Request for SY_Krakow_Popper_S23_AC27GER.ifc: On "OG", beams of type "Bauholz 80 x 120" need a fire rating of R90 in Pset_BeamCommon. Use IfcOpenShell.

First a look at what the model holds.

```python
import ifcopenshell
import ifcopenshell.util.element

model = ifcopenshell.open("SY_Krakow_Popper_S23_AC27GER.ifc")
print(model.schema)
storey = next(s for s in model.by_type("IfcBuildingStorey") if s.Name == "OG")
beams = [e for e in ifcopenshell.util.element.get_decomposition(storey) if e.is_a("IfcBeam")]
seen = {}
for e in beams:
    element_type = ifcopenshell.util.element.get_type(e)
    key = (element_type.Name if element_type != e and element_type else None, ifcopenshell.util.element.get_pset(e, "Pset_BeamCommon", "FireRating"))
    seen[key] = seen.get(key, 0) + 1
for (name, value), count in sorted(seen.items(), key=str):
    print(count, "x", name, "|", value)
```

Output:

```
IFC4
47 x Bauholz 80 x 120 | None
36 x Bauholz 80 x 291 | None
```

```python
import ifcopenshell
import ifcopenshell.api.pset
import ifcopenshell.util.element

model = ifcopenshell.open("SY_Krakow_Popper_S23_AC27GER.ifc")

storey = next(s for s in model.by_type("IfcBuildingStorey") if s.Name == "OG")
beams = [e for e in ifcopenshell.util.element.get_decomposition(storey) if e.is_a("IfcBeam")]

count = 0
for e in beams:
    element_type = ifcopenshell.util.element.get_type(e)
    if element_type in (None, e) or element_type.Name != "Bauholz 80 x 120":
        continue
    # add_pset returns the element's existing set when there is one.
    pset = ifcopenshell.api.pset.add_pset(model, product=e, name="Pset_BeamCommon")
    ifcopenshell.api.pset.edit_pset(model, pset=pset, properties={"FireRating": "R90"})
    count += 1

print(count, "beams updated")

model.write("SY_Krakow_Popper_S23_AC27GER-out.ifc")
```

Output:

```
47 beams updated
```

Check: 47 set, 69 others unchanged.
